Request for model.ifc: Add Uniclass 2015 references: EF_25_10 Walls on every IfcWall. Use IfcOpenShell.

First a look at what the model holds.

```python
import ifcopenshell

model = ifcopenshell.open("model.ifc")
print(model.schema)
print("classifications:", [c.Name for c in model.by_type("IfcClassification")])
for ifc_class in ("IfcDoor", "IfcRoof", "IfcStair", "IfcWall", "IfcWindow"):
    print(ifc_class, len(model.by_type(ifc_class)))
```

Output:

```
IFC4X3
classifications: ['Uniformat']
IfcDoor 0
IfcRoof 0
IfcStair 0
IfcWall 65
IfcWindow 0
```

```python
import ifcopenshell
import ifcopenshell.api.classification

model = ifcopenshell.open("model.ifc")

system = ifcopenshell.api.classification.add_classification(model, classification="Uniclass 2015")

codes = {
    "IfcWall": ("EF_25_10", "Walls"),
}
for ifc_class, (code, name) in codes.items():
    products = model.by_type(ifc_class)
    ifcopenshell.api.classification.add_reference(
        model, products=products, classification=system, identification=code, name=name
    )
    print(code, len(products))

model.write("model-out.ifc")
```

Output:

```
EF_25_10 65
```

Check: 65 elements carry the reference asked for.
